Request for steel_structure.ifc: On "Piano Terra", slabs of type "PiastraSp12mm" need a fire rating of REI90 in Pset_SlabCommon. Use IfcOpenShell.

First a look at what the model holds.

```python
import ifcopenshell
import ifcopenshell.util.element

model = ifcopenshell.open("steel_structure.ifc")
print(model.schema)
storey = next(s for s in model.by_type("IfcBuildingStorey") if s.Name == "Piano Terra")
slabs = [e for e in ifcopenshell.util.element.get_decomposition(storey) if e.is_a("IfcSlab")]
seen = {}
for e in slabs:
    element_type = ifcopenshell.util.element.get_type(e)
    key = (element_type.Name if element_type != e and element_type else None, ifcopenshell.util.element.get_pset(e, "Pset_SlabCommon", "FireRating"))
    seen[key] = seen.get(key, 0) + 1
for (name, value), count in sorted(seen.items(), key=str):
    print(count, "x", name, "|", value)
```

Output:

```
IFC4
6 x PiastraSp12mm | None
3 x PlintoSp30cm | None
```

```python
import ifcopenshell
import ifcopenshell.api.pset
import ifcopenshell.util.element

model = ifcopenshell.open("steel_structure.ifc")

storey = next(s for s in model.by_type("IfcBuildingStorey") if s.Name == "Piano Terra")
slabs = [e for e in ifcopenshell.util.element.get_decomposition(storey) if e.is_a("IfcSlab")]

count = 0
for e in slabs:
    element_type = ifcopenshell.util.element.get_type(e)
    if element_type in (None, e) or element_type.Name != "PiastraSp12mm":
        continue
    # add_pset returns the element's existing set when there is one.
    pset = ifcopenshell.api.pset.add_pset(model, product=e, name="Pset_SlabCommon")
    ifcopenshell.api.pset.edit_pset(model, pset=pset, properties={"FireRating": "REI90"})
    count += 1

print(count, "slabs updated")

model.write("steel_structure_rev.ifc")
```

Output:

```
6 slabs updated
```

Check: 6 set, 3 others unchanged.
